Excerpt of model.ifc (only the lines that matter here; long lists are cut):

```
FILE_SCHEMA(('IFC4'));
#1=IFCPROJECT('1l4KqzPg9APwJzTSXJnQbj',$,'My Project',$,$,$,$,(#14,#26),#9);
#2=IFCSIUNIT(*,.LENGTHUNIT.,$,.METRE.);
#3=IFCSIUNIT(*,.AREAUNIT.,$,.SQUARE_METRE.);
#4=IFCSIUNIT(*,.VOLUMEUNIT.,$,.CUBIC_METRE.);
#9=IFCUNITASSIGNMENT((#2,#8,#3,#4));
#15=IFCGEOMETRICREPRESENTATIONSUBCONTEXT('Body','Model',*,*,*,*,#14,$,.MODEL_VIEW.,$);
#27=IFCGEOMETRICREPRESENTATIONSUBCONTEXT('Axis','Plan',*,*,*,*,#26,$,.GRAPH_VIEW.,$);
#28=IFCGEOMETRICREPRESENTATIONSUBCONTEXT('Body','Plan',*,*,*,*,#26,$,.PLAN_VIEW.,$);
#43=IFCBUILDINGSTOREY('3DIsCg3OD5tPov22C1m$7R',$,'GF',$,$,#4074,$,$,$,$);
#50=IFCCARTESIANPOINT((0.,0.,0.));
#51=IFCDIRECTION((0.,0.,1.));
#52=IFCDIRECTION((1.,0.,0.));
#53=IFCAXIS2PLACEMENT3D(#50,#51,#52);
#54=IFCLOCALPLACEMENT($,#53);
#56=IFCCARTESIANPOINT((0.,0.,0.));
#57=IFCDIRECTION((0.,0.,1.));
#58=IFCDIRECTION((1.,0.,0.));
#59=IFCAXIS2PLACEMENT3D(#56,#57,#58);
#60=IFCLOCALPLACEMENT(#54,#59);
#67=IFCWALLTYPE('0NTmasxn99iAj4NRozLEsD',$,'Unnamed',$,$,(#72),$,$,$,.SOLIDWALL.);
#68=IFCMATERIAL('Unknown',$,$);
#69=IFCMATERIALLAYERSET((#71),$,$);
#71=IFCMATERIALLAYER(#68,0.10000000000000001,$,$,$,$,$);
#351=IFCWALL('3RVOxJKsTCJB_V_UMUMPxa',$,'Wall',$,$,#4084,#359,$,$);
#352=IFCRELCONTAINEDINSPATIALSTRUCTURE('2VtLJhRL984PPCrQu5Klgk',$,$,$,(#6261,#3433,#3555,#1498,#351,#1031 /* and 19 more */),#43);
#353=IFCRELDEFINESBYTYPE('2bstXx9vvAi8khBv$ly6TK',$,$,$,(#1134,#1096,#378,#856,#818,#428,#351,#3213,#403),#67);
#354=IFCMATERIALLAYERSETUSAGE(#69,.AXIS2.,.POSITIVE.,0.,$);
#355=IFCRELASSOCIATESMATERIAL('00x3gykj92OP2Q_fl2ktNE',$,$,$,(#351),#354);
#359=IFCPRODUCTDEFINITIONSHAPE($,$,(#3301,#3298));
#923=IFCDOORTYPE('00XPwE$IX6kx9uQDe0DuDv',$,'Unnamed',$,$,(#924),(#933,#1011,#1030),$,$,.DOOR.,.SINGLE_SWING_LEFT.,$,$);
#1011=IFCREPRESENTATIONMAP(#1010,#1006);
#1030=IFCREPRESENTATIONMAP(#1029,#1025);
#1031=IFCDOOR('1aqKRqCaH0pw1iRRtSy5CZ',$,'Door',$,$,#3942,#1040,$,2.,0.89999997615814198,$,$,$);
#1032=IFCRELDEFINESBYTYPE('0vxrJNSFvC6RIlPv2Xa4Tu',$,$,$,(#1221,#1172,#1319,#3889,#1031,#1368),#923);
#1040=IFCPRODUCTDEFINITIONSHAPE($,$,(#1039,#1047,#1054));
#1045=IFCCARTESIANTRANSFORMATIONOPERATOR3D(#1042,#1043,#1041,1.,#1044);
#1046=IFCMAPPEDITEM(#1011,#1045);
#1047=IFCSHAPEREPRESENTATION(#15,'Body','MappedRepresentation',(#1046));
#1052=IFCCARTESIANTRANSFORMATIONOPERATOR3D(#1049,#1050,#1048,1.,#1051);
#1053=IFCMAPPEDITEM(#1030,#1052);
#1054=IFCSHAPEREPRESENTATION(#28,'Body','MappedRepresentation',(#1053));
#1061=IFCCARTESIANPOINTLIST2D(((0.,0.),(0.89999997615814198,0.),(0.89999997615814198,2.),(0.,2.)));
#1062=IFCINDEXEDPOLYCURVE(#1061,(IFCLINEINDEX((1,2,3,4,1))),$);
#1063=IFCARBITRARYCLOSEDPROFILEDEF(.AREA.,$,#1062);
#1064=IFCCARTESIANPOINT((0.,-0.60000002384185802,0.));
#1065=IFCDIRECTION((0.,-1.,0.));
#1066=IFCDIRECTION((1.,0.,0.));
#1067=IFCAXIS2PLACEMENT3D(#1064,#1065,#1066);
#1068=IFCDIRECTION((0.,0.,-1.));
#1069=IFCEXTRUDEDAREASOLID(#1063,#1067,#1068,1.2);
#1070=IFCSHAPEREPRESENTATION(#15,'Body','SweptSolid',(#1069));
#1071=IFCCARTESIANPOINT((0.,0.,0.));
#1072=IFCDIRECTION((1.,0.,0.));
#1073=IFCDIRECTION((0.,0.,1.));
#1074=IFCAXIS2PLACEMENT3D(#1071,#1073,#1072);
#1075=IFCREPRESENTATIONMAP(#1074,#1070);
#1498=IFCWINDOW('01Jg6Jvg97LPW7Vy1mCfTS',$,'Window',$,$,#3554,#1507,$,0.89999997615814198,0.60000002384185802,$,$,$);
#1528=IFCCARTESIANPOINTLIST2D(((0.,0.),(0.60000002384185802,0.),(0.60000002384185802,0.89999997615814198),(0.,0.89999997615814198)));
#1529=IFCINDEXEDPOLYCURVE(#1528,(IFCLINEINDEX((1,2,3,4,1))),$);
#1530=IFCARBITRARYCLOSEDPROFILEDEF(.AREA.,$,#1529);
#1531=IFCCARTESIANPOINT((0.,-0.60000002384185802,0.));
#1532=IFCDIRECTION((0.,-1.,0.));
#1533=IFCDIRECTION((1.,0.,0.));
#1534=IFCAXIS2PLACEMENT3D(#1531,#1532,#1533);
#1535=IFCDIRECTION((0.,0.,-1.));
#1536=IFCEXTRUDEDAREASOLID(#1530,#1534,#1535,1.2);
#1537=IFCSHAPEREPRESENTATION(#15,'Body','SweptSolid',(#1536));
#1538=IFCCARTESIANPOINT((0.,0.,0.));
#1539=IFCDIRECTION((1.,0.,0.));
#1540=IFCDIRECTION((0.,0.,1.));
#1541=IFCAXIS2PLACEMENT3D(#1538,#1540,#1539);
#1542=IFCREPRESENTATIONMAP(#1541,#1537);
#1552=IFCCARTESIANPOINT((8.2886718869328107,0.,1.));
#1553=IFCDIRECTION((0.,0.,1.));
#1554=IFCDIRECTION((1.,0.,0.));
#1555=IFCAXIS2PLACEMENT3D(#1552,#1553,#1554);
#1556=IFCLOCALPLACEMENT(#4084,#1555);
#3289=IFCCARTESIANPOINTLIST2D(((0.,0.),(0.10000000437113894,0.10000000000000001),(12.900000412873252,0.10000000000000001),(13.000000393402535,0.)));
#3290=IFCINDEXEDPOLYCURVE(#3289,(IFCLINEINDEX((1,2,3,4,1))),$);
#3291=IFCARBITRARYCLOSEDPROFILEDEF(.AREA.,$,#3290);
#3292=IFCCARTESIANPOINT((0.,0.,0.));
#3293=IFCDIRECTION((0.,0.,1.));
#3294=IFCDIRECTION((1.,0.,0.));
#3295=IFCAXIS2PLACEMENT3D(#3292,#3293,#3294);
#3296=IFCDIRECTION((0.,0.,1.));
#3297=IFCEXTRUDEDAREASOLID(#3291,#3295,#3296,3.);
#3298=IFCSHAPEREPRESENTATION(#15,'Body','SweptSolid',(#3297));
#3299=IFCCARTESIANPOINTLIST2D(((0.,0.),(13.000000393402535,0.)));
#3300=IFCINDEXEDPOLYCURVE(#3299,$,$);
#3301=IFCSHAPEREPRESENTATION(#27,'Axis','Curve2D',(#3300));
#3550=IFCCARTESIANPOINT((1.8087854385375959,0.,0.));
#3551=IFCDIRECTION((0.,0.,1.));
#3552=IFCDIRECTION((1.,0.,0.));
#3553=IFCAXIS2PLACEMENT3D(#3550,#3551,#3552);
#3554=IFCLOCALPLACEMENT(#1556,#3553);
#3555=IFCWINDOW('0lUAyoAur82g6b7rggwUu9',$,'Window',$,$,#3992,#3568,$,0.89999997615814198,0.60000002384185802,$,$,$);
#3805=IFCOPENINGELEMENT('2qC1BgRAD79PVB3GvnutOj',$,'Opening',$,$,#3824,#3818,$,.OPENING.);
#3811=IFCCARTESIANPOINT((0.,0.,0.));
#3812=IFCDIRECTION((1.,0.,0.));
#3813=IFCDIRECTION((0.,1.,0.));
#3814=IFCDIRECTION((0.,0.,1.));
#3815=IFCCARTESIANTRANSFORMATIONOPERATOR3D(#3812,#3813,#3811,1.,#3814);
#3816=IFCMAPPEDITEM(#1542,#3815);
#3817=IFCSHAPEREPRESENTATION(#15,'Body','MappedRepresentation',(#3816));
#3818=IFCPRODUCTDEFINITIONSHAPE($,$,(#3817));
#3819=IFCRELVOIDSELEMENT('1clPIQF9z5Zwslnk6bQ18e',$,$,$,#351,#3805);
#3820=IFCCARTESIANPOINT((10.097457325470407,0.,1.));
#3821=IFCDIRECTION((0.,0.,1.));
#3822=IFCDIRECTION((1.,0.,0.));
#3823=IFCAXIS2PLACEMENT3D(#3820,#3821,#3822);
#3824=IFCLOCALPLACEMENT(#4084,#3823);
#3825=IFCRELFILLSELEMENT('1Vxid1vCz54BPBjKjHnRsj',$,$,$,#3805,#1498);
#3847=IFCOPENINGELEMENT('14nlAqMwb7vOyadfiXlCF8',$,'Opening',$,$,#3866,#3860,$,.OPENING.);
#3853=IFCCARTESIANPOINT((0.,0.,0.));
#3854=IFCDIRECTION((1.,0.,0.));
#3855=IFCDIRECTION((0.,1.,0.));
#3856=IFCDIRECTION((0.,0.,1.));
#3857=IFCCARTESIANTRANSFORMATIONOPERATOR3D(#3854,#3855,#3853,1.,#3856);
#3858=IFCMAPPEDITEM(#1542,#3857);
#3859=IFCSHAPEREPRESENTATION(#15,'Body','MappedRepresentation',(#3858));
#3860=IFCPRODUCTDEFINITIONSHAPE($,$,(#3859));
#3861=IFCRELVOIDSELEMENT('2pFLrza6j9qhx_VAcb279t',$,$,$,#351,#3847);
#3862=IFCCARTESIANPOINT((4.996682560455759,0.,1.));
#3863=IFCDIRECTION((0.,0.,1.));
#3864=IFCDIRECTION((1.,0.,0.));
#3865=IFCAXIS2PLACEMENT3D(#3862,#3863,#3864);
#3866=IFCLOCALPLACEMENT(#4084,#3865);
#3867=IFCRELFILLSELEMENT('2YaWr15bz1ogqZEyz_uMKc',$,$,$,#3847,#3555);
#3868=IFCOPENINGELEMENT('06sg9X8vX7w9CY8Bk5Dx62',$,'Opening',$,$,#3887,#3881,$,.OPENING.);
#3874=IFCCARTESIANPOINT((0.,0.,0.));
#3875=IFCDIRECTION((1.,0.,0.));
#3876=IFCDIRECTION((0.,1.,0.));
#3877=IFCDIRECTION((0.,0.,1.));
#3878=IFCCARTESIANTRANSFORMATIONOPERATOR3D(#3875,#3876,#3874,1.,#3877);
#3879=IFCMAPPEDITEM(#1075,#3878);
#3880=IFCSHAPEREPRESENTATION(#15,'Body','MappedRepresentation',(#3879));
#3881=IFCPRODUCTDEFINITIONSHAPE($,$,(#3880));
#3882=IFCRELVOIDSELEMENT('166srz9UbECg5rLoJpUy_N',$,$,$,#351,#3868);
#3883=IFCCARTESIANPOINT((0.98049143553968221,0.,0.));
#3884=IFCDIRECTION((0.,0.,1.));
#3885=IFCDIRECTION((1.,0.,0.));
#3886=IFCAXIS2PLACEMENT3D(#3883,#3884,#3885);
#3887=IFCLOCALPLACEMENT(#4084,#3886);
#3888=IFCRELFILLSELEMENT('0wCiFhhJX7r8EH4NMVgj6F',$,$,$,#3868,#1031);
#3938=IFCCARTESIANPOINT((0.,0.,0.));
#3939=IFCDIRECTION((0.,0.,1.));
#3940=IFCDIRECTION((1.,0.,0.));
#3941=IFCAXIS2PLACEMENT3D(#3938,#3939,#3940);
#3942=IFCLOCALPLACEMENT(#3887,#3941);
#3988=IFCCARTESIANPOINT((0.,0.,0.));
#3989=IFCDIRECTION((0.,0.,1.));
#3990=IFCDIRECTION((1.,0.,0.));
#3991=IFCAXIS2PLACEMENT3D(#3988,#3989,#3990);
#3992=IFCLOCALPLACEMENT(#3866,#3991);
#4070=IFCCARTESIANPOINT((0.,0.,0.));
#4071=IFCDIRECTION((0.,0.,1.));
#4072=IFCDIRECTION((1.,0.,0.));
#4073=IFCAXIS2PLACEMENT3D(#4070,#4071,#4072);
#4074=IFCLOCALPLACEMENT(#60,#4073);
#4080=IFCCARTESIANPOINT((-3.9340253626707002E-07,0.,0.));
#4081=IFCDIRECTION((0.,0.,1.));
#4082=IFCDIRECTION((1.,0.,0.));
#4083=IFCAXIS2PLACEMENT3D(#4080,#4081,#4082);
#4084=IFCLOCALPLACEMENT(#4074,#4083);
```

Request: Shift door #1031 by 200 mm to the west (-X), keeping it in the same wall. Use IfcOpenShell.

```python
import ifcopenshell
import ifcopenshell.api.geometry
import ifcopenshell.util.placement
import ifcopenshell.util.unit

model = ifcopenshell.open("model.ifc")
unit_scale = ifcopenshell.util.unit.calculate_unit_scale(model)

door = model.by_id(1031)
opening = door.FillsVoids[0].RelatingOpeningElement
wall = opening.VoidsElements[0].RelatingBuildingElement

wall_matrix = ifcopenshell.util.placement.get_local_placement(wall.ObjectPlacement)
shift = wall_matrix[:3, 0] * -0.2 / unit_scale
before = ifcopenshell.util.placement.get_local_placement(door.ObjectPlacement)[:3, 3].copy()

# The door is placed relative to its opening, so it follows when the opening moves.
matrix = ifcopenshell.util.placement.get_local_placement(opening.ObjectPlacement)
matrix[:3, 3] += shift
ifcopenshell.api.geometry.edit_object_placement(
    model, product=opening, matrix=matrix, is_si=False, should_transform_children=True
)

after = ifcopenshell.util.placement.get_local_placement(door.ObjectPlacement)[:3, 3]
print("door moved by", (after - before).round(3) + 0.0)

model.write("model_v2.ifc")
```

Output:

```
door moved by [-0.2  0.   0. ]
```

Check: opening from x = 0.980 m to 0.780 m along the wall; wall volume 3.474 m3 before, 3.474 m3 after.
